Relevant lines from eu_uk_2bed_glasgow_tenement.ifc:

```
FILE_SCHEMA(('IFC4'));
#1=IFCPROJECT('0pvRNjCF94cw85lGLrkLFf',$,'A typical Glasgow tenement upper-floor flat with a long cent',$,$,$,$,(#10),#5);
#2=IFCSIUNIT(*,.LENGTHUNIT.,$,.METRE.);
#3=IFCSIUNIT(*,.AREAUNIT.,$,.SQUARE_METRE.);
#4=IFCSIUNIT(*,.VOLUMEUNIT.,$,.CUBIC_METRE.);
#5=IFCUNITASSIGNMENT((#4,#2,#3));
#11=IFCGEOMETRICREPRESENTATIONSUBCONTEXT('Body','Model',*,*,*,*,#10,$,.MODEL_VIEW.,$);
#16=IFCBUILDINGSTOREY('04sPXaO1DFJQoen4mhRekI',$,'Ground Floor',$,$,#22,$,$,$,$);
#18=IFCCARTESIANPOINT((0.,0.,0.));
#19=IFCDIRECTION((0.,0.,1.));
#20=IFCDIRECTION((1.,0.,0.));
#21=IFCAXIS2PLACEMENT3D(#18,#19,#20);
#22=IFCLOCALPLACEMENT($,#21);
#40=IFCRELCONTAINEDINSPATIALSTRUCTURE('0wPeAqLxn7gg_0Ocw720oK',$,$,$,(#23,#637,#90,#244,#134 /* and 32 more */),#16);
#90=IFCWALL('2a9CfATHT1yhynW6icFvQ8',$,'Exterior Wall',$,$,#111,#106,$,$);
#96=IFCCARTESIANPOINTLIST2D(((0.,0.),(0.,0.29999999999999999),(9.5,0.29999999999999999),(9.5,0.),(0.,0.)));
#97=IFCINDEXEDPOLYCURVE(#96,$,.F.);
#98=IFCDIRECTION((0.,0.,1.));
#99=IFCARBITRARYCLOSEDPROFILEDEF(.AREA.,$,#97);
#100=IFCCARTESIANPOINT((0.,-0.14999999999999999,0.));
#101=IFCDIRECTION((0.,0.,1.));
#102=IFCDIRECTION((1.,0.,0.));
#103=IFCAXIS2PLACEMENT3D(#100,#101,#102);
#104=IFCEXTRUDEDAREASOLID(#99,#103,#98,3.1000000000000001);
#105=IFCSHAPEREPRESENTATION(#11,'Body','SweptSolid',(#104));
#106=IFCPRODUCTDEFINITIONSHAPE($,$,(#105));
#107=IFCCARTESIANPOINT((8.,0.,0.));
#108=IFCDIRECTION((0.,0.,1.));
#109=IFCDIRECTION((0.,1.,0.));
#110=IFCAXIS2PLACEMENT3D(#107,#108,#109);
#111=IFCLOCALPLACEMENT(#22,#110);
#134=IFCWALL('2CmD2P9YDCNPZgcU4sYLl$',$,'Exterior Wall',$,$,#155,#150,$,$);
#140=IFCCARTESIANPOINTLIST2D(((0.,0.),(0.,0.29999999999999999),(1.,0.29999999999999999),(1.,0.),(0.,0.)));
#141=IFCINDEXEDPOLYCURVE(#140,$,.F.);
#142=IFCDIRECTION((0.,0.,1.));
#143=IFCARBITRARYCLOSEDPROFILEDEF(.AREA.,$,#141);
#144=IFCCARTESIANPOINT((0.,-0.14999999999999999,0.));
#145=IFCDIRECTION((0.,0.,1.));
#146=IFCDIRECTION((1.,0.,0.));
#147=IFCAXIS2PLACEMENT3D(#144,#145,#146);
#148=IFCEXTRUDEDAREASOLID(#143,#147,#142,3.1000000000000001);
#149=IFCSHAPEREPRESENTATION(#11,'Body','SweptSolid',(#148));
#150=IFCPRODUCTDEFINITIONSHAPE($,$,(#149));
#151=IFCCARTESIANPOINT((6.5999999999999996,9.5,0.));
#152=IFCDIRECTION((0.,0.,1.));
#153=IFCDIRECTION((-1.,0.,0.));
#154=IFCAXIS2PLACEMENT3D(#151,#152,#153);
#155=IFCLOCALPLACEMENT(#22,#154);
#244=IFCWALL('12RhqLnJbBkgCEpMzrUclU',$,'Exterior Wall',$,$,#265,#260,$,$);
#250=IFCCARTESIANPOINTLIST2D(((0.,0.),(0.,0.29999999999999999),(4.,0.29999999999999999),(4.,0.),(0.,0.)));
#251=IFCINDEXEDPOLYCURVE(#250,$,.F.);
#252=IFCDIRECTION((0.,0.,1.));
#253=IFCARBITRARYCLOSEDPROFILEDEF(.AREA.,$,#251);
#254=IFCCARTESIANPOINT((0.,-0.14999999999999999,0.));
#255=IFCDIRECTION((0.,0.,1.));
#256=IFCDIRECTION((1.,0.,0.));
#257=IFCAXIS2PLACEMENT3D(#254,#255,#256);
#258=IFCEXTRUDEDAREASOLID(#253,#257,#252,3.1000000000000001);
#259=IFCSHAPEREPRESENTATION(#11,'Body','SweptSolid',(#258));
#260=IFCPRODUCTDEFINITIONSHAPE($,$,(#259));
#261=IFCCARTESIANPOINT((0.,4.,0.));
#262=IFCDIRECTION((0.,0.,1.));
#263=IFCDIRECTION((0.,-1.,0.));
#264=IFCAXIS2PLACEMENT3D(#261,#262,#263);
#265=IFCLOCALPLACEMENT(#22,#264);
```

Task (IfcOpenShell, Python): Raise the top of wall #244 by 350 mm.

```python
import ifcopenshell
import ifcopenshell.geom
import ifcopenshell.util.representation
import ifcopenshell.util.shape
import ifcopenshell.util.unit

model = ifcopenshell.open("eu_uk_2bed_glasgow_tenement.ifc")
unit_scale = ifcopenshell.util.unit.calculate_unit_scale(model)
settings = ifcopenshell.geom.settings()


def volume(element):
    """Net volume in cubic metres, openings subtracted."""
    shape = ifcopenshell.geom.create_shape(settings, element)
    return ifcopenshell.util.shape.get_volume(shape.geometry)


wall = model.by_id(244)
before = volume(wall)

body = ifcopenshell.util.representation.get_representation(wall, "Model", "Body")
solid = body.Items[0]
old_height = solid.Depth
solid.Depth += 0.35 / unit_scale
after = volume(wall)

print(f"height {old_height:g} -> {solid.Depth:g}, volume {before:.3f} -> {after:.3f} m3")

model.write("eu_uk_2bed_glasgow_tenement_v2.ifc")
```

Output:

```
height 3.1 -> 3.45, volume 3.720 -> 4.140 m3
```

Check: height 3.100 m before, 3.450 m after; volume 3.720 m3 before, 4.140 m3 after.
